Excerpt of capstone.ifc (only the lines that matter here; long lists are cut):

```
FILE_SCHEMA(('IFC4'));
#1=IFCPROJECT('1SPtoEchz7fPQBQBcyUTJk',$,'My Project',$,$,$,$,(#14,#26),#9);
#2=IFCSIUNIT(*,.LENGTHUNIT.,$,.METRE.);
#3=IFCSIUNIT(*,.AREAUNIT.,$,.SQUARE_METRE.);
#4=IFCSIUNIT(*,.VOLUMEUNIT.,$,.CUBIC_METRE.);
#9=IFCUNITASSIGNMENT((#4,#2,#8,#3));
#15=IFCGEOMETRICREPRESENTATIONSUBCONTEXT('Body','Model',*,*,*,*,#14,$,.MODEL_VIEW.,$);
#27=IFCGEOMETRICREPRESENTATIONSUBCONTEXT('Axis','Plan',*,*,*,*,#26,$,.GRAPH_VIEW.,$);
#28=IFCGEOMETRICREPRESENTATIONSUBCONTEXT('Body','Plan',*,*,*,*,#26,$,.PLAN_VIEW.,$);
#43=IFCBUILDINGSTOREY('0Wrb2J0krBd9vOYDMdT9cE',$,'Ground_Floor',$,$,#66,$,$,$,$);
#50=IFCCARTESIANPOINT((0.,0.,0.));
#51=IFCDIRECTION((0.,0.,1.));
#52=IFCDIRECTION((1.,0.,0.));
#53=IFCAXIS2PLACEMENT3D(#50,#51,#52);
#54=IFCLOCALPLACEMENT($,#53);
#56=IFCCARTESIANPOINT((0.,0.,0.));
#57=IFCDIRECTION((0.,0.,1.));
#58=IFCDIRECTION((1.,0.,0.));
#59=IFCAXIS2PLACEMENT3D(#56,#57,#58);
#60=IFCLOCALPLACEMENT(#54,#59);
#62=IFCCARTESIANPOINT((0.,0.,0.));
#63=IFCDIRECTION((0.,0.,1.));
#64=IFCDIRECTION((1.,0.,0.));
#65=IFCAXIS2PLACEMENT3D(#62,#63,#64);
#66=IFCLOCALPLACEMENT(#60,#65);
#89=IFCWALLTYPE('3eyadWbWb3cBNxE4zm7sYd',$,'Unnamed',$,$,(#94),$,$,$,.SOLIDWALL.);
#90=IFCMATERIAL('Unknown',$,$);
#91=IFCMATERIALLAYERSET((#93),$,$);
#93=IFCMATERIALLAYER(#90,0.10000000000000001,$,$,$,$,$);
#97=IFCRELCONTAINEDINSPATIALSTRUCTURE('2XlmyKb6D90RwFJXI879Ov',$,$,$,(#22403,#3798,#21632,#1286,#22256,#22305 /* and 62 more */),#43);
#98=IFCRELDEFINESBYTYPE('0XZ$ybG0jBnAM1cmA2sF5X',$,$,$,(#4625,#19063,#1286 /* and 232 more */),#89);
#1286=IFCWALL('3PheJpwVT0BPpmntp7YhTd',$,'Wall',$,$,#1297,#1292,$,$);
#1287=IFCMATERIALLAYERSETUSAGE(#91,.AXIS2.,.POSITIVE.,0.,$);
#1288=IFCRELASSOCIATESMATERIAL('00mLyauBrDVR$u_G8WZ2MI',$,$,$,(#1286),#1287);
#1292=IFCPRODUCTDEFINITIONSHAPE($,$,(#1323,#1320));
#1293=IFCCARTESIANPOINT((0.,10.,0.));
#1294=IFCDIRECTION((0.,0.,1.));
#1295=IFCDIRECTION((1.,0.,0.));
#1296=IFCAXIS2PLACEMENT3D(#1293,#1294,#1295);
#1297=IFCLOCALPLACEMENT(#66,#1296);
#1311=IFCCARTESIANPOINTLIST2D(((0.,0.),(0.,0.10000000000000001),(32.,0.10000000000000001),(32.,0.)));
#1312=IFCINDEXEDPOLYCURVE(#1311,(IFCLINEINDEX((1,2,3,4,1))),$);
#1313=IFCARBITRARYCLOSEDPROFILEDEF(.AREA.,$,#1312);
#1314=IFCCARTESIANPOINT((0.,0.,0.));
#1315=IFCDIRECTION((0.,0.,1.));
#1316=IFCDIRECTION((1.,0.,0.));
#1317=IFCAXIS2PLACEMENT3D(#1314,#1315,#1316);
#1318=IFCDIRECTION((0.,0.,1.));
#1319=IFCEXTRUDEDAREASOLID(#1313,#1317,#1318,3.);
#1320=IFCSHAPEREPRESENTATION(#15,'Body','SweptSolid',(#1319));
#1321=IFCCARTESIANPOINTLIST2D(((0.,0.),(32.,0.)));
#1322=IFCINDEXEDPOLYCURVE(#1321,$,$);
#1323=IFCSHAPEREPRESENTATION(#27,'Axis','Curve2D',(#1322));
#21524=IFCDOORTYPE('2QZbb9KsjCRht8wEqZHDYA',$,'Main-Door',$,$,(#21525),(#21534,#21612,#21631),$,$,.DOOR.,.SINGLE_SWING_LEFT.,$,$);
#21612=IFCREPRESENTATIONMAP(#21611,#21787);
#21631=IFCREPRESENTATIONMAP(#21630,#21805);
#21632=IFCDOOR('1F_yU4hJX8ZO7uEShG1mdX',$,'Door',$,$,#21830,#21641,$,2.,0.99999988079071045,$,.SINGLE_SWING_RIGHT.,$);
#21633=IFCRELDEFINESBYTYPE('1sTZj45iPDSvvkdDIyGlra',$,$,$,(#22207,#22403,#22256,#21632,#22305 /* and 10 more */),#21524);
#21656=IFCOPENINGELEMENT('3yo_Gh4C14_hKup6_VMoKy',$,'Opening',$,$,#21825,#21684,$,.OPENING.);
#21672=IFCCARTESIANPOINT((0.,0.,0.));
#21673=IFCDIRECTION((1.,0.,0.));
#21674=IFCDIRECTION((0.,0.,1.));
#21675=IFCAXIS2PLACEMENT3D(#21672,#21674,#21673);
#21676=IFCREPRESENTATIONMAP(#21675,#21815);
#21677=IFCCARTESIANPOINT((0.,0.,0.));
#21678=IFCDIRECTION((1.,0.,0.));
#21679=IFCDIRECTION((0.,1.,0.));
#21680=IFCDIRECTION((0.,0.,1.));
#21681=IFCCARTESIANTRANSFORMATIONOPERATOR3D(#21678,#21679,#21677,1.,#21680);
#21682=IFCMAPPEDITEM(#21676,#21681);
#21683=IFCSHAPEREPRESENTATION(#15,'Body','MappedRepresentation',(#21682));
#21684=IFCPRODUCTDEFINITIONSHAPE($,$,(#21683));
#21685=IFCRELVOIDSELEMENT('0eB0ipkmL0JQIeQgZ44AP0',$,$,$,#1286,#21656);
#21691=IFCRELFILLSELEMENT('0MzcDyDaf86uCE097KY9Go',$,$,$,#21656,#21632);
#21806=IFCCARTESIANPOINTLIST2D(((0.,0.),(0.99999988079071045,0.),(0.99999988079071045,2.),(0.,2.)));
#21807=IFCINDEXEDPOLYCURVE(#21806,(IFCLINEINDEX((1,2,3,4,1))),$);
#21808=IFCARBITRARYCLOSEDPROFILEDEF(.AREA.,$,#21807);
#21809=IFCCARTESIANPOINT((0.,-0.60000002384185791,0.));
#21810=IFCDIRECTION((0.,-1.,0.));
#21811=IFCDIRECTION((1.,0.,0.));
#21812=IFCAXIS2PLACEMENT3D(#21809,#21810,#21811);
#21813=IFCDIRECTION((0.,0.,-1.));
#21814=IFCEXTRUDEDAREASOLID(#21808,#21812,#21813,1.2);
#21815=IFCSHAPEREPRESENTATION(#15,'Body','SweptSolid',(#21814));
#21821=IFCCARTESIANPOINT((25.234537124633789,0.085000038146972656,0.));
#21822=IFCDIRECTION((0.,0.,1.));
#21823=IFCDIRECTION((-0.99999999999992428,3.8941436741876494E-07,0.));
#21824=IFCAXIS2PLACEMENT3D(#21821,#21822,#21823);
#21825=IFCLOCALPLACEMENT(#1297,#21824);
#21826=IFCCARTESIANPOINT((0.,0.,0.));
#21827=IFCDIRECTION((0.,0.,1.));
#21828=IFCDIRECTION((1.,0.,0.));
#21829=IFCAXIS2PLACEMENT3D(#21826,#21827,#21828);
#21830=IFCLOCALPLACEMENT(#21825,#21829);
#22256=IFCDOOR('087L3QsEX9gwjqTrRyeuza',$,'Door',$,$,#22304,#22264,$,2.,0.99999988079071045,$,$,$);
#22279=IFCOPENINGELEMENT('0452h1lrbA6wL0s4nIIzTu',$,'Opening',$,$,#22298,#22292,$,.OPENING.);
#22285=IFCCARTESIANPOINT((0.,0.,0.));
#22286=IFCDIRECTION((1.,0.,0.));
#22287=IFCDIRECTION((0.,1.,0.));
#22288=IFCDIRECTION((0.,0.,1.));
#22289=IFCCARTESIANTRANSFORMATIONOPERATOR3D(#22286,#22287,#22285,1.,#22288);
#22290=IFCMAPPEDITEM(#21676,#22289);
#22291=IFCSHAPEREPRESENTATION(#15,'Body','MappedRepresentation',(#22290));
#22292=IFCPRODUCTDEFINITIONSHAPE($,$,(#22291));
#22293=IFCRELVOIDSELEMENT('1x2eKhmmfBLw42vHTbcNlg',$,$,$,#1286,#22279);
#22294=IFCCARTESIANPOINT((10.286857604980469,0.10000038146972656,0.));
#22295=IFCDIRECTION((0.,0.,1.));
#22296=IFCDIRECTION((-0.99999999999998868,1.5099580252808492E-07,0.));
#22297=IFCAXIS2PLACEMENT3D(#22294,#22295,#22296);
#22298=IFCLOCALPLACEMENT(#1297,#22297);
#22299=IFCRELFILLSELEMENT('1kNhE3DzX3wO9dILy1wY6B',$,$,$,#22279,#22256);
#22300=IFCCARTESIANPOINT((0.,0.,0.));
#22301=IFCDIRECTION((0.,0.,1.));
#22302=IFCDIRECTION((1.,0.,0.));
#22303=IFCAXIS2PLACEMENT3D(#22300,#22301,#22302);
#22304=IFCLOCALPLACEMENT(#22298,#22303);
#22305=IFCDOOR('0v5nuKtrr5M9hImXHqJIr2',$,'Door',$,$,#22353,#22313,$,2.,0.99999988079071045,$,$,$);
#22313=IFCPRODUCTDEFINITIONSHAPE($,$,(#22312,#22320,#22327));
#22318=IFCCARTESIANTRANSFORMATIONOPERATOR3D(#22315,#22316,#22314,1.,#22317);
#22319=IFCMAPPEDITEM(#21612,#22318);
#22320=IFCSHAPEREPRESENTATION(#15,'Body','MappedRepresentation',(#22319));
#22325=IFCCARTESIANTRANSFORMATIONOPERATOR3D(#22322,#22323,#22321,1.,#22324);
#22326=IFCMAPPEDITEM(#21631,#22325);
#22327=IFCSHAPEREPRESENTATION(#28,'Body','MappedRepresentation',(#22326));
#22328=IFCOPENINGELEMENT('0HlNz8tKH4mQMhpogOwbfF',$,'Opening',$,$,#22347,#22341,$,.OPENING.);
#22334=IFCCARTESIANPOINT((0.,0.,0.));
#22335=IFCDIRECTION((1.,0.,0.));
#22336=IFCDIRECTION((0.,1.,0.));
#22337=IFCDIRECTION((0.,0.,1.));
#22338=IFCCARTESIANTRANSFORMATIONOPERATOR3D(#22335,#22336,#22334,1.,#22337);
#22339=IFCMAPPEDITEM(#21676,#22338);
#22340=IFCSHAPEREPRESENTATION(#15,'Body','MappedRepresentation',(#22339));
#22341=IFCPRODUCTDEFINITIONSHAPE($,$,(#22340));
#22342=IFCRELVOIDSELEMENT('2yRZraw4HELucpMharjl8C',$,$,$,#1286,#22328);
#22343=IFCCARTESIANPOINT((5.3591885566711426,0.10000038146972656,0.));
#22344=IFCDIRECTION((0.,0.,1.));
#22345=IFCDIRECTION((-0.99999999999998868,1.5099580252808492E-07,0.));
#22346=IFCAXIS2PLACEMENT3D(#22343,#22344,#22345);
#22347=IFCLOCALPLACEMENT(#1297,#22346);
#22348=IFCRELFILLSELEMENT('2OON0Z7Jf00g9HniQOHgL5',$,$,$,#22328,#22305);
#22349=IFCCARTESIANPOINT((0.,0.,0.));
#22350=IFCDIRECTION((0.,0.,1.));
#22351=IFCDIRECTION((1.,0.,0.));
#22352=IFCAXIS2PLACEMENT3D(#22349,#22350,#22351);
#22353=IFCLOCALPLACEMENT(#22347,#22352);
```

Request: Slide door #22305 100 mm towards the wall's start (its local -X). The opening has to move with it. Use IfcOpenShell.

```python
import ifcopenshell
import ifcopenshell.api.geometry
import ifcopenshell.util.placement

model = ifcopenshell.open("capstone.ifc")

door = model.by_id(22305)
opening = door.FillsVoids[0].RelatingOpeningElement
wall = opening.VoidsElements[0].RelatingBuildingElement

wall_matrix = ifcopenshell.util.placement.get_local_placement(wall.ObjectPlacement)
shift = wall_matrix[:3, 0] * -0.1
before = ifcopenshell.util.placement.get_local_placement(door.ObjectPlacement)[:3, 3].copy()

# The door is placed relative to its opening, so it follows when the opening moves.
matrix = ifcopenshell.util.placement.get_local_placement(opening.ObjectPlacement)
matrix[:3, 3] += shift
ifcopenshell.api.geometry.edit_object_placement(
    model, product=opening, matrix=matrix, is_si=False, should_transform_children=True
)

after = ifcopenshell.util.placement.get_local_placement(door.ObjectPlacement)[:3, 3]
print("door moved by", (after - before).round(3) + 0.0)

model.write("capstone_updated.ifc")
```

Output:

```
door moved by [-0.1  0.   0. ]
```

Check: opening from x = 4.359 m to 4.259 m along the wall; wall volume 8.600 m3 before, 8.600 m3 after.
